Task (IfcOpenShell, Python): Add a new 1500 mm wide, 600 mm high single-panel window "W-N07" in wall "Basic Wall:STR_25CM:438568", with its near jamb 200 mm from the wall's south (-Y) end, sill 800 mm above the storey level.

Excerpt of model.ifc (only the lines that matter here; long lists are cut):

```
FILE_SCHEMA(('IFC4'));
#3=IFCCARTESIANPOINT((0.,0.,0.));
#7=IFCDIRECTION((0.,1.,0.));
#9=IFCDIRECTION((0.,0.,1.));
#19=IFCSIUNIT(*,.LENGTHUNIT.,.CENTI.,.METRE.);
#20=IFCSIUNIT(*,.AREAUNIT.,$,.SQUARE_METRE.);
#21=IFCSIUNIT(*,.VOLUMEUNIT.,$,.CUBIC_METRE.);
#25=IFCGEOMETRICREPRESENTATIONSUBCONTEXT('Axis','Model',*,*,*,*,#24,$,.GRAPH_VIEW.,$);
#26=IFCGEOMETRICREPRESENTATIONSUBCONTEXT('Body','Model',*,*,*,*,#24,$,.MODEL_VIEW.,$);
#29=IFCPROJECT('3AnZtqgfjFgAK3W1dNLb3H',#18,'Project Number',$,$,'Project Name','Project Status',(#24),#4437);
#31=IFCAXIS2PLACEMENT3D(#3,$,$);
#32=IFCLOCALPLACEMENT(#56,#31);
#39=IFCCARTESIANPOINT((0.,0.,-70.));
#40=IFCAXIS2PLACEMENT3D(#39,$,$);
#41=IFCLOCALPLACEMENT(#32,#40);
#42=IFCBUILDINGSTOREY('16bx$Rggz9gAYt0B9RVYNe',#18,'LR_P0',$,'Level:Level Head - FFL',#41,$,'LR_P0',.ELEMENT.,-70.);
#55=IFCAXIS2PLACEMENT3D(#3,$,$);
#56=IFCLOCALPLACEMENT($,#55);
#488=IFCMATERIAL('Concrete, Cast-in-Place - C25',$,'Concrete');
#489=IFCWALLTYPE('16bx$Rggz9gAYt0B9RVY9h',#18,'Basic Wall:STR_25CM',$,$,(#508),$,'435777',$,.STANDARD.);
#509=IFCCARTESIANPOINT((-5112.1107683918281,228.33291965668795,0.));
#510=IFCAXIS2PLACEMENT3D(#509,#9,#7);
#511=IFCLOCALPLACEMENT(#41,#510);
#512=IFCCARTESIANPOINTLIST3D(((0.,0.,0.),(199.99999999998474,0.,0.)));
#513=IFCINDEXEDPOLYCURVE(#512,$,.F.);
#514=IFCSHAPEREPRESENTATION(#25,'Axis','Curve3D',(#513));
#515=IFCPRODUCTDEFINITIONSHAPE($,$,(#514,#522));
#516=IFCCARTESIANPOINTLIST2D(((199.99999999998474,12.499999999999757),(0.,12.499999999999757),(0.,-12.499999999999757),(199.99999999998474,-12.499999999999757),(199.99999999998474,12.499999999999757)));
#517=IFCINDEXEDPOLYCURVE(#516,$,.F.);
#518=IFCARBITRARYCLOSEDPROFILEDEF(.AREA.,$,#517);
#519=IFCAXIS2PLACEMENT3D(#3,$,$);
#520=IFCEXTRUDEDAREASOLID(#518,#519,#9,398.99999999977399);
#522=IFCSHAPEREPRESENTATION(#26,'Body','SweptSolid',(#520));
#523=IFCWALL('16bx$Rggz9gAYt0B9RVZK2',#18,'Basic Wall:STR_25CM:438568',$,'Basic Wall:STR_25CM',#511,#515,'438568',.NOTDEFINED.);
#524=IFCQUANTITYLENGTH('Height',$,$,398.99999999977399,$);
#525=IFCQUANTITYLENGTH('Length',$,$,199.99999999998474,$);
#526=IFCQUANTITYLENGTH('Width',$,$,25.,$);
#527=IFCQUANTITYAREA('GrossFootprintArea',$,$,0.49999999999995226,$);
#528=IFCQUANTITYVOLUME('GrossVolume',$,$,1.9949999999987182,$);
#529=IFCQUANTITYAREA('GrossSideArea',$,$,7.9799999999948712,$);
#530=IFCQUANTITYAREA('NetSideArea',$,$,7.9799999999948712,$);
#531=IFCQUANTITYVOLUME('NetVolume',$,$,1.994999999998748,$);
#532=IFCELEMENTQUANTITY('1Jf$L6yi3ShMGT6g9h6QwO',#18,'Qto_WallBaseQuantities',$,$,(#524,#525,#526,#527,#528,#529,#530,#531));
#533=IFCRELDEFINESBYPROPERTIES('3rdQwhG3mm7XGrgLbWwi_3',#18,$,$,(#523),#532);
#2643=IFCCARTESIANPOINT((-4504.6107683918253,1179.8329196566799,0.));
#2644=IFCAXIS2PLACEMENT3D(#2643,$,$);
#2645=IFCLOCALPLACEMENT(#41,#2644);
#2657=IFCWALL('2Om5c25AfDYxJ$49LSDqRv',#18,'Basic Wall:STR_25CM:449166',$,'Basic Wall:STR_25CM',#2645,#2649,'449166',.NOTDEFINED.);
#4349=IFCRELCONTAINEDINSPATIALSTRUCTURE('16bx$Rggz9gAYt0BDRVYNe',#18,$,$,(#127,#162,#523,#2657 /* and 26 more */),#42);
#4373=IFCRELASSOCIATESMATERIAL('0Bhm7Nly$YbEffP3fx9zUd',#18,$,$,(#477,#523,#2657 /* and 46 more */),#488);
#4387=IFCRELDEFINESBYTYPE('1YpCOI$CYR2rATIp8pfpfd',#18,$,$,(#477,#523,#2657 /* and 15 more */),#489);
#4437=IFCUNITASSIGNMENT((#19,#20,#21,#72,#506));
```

```python
import numpy as np
import ifcopenshell
import ifcopenshell.api.feature
import ifcopenshell.api.geometry
import ifcopenshell.api.pset
import ifcopenshell.api.root
import ifcopenshell.api.spatial
import ifcopenshell.geom
import ifcopenshell.util.element
import ifcopenshell.util.placement
import ifcopenshell.util.representation
import ifcopenshell.util.shape
import ifcopenshell.util.unit

model = ifcopenshell.open("model.ifc")
unit_scale = ifcopenshell.util.unit.calculate_unit_scale(model)
area_scale = ifcopenshell.util.unit.calculate_unit_scale(model, "AREAUNIT")
volume_scale = ifcopenshell.util.unit.calculate_unit_scale(model, "VOLUMEUNIT")
settings = ifcopenshell.geom.settings()


def volume(element):
    """Net volume in cubic metres, openings subtracted."""
    shape = ifcopenshell.geom.create_shape(settings, element)
    return ifcopenshell.util.shape.get_volume(shape.geometry)


wall = model.by_guid("16bx$Rggz9gAYt0B9RVZK2")
storey = ifcopenshell.util.element.get_container(wall, ifc_class="IfcBuildingStorey")
context = ifcopenshell.util.representation.get_context(model, "Model", "Body", "MODEL_VIEW")
before = volume(wall)

width, height, from_end, sill = 1.5, 0.6, 0.2, 0.8  # metres

# The wall runs along its own X axis, and the end named is its -X end.
wall_shape = ifcopenshell.geom.create_shape(settings, wall)
x, y, z = ifcopenshell.util.shape.get_vertices(wall_shape.geometry).T
start = x.min() + from_end
face, thickness = float(y.min()), float(y.max() - y.min())
wall_matrix = ifcopenshell.util.placement.get_local_placement(wall.ObjectPlacement)
level = ifcopenshell.util.placement.get_local_placement(storey.ObjectPlacement)[2, 3]


def in_wall(x, y):
    """Placement at x, y metres in the wall's axes, at sill height."""
    matrix = wall_matrix.copy()
    matrix[:, 3] = wall_matrix @ np.array([x / unit_scale, y / unit_scale, 0.0, 1.0])
    matrix[2, 3] = level + sill / unit_scale
    return matrix


# Opening: a box that overshoots both wall faces by 50 mm.
opening = ifcopenshell.api.root.create_entity(model, ifc_class="IfcOpeningElement", predefined_type="OPENING")
box = ifcopenshell.api.geometry.add_wall_representation(
    model, context=context, length=width, height=height, thickness=thickness + 0.1
)
ifcopenshell.api.geometry.assign_representation(model, product=opening, representation=box)
ifcopenshell.api.geometry.edit_object_placement(model, product=opening, matrix=in_wall(start, face - 0.05), is_si=False)
ifcopenshell.api.feature.add_feature(model, feature=opening, element=wall)

window = ifcopenshell.api.root.create_entity(model, ifc_class="IfcWindow", name="W-N07", predefined_type="WINDOW")
window.OverallWidth, window.OverallHeight = width / unit_scale, height / unit_scale
window.PartitioningType = "SINGLE_PANEL"
body = ifcopenshell.api.geometry.add_window_representation(
    model,
    context=context,
    overall_width=window.OverallWidth,
    overall_height=window.OverallHeight,
    partition_type="SINGLE_PANEL",
)
ifcopenshell.api.geometry.assign_representation(model, product=window, representation=body)
ifcopenshell.api.spatial.assign_container(model, products=[window], relating_structure=storey)
ifcopenshell.api.feature.add_filling(model, opening=opening, element=window)

# Centre the window in the wall's thickness.
ifcopenshell.api.geometry.edit_object_placement(model, product=window, matrix=in_wall(start, face), is_si=False)
window_shape = ifcopenshell.geom.create_shape(settings, window)
depth = ifcopenshell.util.shape.get_vertices(window_shape.geometry)[:, 1]
offset = face + thickness / 2 - (depth.min() + depth.max()) / 2
ifcopenshell.api.geometry.edit_object_placement(model, product=window, matrix=in_wall(start, offset), is_si=False)

after = volume(wall)

# Update the wall's stored quantities.
qto = model.by_id(ifcopenshell.util.element.get_pset(wall, "Qto_WallBaseQuantities", should_inherit=False)["id"])
ifcopenshell.api.pset.edit_qto(model, qto=qto, properties={
    "NetSideArea": after / thickness / area_scale,
    "NetVolume": after / volume_scale,
})

print(f"wall volume {before:.3f} -> {after:.3f} m3")

model.write("model_updated.ifc")
```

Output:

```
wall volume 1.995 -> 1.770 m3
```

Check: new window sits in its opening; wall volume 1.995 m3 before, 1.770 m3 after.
